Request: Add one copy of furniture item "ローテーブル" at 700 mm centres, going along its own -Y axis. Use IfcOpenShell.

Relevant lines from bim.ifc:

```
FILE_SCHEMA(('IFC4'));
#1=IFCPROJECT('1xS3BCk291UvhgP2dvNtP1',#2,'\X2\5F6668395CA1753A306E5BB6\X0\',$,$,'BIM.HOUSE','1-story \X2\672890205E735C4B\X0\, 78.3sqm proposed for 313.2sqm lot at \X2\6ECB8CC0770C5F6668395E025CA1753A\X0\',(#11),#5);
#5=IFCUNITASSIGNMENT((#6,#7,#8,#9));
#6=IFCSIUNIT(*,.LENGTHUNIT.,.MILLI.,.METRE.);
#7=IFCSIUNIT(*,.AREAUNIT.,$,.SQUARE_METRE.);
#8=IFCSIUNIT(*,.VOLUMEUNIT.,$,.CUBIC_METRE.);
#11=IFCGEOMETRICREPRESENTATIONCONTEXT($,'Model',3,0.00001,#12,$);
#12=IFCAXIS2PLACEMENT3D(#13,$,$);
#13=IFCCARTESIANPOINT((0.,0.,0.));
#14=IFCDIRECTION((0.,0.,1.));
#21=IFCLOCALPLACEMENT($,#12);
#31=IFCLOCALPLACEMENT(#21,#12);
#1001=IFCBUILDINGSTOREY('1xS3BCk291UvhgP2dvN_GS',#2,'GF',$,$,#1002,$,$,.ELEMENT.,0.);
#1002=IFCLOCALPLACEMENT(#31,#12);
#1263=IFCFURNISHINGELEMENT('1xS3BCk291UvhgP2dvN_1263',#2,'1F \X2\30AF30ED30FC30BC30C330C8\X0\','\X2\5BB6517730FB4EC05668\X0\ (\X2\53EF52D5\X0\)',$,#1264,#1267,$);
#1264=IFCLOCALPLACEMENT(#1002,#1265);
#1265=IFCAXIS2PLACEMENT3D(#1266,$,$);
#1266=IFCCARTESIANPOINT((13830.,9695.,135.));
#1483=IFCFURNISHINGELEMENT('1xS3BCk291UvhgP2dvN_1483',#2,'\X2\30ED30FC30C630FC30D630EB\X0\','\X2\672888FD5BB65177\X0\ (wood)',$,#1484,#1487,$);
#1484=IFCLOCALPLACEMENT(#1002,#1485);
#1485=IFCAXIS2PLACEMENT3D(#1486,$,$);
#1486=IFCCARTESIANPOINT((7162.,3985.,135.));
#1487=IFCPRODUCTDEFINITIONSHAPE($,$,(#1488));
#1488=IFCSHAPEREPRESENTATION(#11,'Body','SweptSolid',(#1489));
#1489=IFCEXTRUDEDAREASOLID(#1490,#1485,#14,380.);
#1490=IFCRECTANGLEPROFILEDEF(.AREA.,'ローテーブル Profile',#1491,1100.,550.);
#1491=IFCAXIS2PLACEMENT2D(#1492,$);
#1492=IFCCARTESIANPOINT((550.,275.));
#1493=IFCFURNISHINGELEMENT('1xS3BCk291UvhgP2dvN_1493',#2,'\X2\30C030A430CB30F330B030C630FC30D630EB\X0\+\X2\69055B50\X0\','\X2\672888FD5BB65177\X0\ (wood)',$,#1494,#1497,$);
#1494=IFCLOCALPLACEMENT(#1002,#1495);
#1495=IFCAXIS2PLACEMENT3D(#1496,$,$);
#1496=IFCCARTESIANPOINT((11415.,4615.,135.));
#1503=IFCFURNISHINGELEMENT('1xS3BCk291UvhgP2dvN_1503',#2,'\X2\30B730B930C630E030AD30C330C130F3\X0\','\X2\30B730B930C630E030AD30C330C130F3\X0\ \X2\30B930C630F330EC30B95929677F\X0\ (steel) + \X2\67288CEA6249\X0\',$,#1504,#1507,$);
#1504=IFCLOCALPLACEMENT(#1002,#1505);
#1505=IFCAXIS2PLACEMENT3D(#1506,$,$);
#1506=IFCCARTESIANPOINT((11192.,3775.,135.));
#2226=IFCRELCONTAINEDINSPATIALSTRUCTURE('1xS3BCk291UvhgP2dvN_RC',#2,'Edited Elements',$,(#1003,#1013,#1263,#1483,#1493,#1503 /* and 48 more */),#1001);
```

```python
import ifcopenshell
import ifcopenshell.api.geometry
import ifcopenshell.api.root
import ifcopenshell.util.element
import ifcopenshell.util.placement

model = ifcopenshell.open("bim.ifc")


def reuse_history(source, copy):
    """copy_class also copies each property set's owner history, people and application; keep the originals."""
    for rel in copy.IsDefinedBy:
        if rel.is_a("IfcRelDefinesByProperties") and (history := rel.RelatingPropertyDefinition.OwnerHistory):
            rel.RelatingPropertyDefinition.OwnerHistory = source.OwnerHistory
            ifcopenshell.util.element.remove_deep2(model, history)


source = model.by_guid("1xS3BCk291UvhgP2dvN_1483")
base = ifcopenshell.util.placement.get_local_placement(source.ObjectPlacement)
step = -base[:3, 1] * 700.0

for i in range(1, 2):
    copy = ifcopenshell.api.root.copy_class(model, product=source)
    copy.Representation = ifcopenshell.util.element.copy_deep(
        model, source.Representation, exclude=["IfcGeometricRepresentationContext", "IfcRepresentationMap"]
    )
    reuse_history(source, copy)
    matrix = base.copy()
    matrix[:3, 3] += i * step
    print("added at", matrix[:3, 3].round(3) + 0.0)
    ifcopenshell.api.geometry.edit_object_placement(model, product=copy, matrix=matrix, is_si=False)

model.write("bim_updated.ifc")
```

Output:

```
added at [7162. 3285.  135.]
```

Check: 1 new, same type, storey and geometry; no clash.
